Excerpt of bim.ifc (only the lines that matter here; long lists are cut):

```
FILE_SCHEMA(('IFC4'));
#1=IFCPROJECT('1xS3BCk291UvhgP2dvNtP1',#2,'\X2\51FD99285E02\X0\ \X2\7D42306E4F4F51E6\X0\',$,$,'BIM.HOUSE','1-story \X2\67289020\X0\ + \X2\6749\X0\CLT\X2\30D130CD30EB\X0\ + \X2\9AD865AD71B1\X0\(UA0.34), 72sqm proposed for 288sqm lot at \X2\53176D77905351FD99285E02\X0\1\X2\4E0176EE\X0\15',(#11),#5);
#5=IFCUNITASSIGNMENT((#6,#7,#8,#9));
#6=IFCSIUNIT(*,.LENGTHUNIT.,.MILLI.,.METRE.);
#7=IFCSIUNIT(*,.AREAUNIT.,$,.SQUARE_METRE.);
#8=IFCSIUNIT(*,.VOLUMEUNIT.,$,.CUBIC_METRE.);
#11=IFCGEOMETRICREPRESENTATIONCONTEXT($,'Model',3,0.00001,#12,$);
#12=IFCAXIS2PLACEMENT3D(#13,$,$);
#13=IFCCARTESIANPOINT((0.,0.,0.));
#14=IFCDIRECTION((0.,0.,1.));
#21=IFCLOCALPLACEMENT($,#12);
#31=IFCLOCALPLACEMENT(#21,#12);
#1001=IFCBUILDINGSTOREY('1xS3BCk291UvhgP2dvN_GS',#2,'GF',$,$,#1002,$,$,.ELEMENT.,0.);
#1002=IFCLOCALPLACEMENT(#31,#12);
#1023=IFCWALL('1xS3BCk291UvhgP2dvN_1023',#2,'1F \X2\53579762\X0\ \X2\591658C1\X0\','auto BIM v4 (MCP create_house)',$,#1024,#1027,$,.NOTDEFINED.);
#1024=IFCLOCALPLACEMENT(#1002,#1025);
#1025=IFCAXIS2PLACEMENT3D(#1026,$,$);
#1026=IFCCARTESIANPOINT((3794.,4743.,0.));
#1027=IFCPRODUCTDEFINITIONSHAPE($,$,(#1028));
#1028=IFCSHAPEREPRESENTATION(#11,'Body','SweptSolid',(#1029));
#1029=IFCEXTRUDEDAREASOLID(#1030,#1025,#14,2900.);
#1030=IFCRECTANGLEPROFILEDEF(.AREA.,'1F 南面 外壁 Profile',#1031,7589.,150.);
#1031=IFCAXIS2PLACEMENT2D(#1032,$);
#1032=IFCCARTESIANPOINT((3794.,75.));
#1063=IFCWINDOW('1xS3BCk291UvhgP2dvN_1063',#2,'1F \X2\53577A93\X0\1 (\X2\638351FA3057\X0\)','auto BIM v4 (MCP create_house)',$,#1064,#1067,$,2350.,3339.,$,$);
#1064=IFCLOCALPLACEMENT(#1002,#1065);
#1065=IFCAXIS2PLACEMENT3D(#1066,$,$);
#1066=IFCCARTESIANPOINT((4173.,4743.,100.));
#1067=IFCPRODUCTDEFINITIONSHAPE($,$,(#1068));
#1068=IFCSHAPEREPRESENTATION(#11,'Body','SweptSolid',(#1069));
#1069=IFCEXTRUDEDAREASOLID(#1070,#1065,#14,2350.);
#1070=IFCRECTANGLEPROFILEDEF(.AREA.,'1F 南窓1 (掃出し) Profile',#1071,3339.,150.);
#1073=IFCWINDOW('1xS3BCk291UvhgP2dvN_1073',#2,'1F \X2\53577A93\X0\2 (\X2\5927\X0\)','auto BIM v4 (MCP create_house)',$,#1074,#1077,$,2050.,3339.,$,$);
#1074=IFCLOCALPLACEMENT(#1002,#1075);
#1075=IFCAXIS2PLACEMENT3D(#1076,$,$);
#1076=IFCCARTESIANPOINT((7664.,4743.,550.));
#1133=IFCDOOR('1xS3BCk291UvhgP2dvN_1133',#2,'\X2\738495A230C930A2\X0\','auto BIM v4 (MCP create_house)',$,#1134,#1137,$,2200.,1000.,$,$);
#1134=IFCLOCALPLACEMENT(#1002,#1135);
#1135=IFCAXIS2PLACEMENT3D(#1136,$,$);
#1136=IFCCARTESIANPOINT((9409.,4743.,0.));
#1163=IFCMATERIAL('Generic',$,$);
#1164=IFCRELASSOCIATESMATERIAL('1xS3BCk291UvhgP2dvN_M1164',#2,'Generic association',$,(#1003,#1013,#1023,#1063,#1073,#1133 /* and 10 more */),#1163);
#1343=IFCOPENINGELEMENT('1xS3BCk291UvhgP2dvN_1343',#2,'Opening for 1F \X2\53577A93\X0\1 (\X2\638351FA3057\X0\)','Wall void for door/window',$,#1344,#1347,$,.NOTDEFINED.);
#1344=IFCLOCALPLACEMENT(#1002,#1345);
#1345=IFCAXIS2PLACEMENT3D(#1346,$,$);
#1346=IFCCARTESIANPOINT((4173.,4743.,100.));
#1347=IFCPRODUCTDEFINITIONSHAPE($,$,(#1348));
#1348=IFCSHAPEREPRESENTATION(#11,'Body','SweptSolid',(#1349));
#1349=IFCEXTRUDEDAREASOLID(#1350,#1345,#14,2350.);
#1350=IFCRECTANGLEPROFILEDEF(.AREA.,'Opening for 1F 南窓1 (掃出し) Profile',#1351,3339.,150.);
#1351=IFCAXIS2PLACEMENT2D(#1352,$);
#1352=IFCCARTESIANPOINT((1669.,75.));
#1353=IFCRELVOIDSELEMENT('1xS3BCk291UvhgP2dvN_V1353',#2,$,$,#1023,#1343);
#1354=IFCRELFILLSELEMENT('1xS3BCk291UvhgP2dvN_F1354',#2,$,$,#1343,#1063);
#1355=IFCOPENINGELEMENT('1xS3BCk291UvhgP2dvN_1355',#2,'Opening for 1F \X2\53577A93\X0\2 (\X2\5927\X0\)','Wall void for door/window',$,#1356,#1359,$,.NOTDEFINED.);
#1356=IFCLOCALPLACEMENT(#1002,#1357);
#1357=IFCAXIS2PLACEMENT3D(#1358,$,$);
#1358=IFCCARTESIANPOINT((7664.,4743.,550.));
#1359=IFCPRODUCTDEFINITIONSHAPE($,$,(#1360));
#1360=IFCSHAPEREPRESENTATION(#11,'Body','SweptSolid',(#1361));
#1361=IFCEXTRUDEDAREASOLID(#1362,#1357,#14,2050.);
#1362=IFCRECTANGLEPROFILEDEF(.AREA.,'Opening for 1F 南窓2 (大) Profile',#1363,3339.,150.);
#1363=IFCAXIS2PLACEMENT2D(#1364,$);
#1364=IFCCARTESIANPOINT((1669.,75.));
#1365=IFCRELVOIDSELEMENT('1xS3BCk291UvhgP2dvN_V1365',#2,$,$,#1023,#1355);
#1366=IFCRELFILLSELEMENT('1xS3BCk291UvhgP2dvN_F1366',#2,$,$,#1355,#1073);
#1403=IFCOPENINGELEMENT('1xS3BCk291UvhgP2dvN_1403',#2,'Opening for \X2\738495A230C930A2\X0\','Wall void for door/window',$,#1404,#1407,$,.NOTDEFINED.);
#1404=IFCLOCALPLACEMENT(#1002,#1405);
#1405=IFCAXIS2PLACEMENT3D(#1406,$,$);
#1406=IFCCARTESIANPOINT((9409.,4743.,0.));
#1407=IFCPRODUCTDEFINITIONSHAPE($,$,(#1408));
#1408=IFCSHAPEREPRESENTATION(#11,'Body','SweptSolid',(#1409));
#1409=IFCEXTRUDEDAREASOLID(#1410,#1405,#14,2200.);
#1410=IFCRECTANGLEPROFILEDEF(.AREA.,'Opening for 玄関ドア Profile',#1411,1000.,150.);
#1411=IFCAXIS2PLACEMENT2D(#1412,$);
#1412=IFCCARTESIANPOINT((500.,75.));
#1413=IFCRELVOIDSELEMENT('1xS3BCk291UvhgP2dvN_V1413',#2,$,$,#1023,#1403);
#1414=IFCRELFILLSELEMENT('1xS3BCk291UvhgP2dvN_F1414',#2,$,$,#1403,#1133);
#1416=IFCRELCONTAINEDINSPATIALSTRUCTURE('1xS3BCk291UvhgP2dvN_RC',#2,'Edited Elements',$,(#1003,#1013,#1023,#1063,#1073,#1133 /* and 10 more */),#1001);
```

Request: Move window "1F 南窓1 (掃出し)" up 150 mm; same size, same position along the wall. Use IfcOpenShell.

```python
import numpy as np
import ifcopenshell
import ifcopenshell.api.geometry
import ifcopenshell.util.placement
import ifcopenshell.util.unit

model = ifcopenshell.open("bim.ifc")
unit_scale = ifcopenshell.util.unit.calculate_unit_scale(model)

window = model.by_guid("1xS3BCk291UvhgP2dvN_1063")
opening = window.FillsVoids[0].RelatingOpeningElement
dz = 0.15 / unit_scale

shift = np.array([0.0, 0.0, dz])
# The window is not placed relative to its opening, so move both.
for product in (opening, window):
    matrix = ifcopenshell.util.placement.get_local_placement(product.ObjectPlacement)
    matrix[:3, 3] += shift
    ifcopenshell.api.geometry.edit_object_placement(model, product=product, matrix=matrix, is_si=False)

print(f"moved by {dz * unit_scale:+.3f} m")

model.write("bim_updated.ifc")
```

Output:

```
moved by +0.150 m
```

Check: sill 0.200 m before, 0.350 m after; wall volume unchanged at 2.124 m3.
